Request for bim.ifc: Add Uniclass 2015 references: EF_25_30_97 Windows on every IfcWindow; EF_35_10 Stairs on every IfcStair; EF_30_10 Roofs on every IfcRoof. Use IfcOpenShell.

First a look at what the model holds.

```python
import ifcopenshell

model = ifcopenshell.open("bim.ifc")
print(model.schema)
print("classifications:", [c.Name for c in model.by_type("IfcClassification")])
for ifc_class in ("IfcDoor", "IfcRoof", "IfcStair", "IfcWall", "IfcWindow"):
    print(ifc_class, len(model.by_type(ifc_class)))
```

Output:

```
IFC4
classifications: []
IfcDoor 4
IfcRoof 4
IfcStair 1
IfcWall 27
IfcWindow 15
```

```python
import ifcopenshell
import ifcopenshell.api.classification

model = ifcopenshell.open("bim.ifc")

system = ifcopenshell.api.classification.add_classification(model, classification="Uniclass 2015")

codes = {
    "IfcWindow": ("EF_25_30_97", "Windows"),
    "IfcStair": ("EF_35_10", "Stairs"),
    "IfcRoof": ("EF_30_10", "Roofs"),
}
for ifc_class, (code, name) in codes.items():
    products = model.by_type(ifc_class)
    ifcopenshell.api.classification.add_reference(
        model, products=products, classification=system, identification=code, name=name
    )
    print(code, len(products))

model.write("bim_rev.ifc")
```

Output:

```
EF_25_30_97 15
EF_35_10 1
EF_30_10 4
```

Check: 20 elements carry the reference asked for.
